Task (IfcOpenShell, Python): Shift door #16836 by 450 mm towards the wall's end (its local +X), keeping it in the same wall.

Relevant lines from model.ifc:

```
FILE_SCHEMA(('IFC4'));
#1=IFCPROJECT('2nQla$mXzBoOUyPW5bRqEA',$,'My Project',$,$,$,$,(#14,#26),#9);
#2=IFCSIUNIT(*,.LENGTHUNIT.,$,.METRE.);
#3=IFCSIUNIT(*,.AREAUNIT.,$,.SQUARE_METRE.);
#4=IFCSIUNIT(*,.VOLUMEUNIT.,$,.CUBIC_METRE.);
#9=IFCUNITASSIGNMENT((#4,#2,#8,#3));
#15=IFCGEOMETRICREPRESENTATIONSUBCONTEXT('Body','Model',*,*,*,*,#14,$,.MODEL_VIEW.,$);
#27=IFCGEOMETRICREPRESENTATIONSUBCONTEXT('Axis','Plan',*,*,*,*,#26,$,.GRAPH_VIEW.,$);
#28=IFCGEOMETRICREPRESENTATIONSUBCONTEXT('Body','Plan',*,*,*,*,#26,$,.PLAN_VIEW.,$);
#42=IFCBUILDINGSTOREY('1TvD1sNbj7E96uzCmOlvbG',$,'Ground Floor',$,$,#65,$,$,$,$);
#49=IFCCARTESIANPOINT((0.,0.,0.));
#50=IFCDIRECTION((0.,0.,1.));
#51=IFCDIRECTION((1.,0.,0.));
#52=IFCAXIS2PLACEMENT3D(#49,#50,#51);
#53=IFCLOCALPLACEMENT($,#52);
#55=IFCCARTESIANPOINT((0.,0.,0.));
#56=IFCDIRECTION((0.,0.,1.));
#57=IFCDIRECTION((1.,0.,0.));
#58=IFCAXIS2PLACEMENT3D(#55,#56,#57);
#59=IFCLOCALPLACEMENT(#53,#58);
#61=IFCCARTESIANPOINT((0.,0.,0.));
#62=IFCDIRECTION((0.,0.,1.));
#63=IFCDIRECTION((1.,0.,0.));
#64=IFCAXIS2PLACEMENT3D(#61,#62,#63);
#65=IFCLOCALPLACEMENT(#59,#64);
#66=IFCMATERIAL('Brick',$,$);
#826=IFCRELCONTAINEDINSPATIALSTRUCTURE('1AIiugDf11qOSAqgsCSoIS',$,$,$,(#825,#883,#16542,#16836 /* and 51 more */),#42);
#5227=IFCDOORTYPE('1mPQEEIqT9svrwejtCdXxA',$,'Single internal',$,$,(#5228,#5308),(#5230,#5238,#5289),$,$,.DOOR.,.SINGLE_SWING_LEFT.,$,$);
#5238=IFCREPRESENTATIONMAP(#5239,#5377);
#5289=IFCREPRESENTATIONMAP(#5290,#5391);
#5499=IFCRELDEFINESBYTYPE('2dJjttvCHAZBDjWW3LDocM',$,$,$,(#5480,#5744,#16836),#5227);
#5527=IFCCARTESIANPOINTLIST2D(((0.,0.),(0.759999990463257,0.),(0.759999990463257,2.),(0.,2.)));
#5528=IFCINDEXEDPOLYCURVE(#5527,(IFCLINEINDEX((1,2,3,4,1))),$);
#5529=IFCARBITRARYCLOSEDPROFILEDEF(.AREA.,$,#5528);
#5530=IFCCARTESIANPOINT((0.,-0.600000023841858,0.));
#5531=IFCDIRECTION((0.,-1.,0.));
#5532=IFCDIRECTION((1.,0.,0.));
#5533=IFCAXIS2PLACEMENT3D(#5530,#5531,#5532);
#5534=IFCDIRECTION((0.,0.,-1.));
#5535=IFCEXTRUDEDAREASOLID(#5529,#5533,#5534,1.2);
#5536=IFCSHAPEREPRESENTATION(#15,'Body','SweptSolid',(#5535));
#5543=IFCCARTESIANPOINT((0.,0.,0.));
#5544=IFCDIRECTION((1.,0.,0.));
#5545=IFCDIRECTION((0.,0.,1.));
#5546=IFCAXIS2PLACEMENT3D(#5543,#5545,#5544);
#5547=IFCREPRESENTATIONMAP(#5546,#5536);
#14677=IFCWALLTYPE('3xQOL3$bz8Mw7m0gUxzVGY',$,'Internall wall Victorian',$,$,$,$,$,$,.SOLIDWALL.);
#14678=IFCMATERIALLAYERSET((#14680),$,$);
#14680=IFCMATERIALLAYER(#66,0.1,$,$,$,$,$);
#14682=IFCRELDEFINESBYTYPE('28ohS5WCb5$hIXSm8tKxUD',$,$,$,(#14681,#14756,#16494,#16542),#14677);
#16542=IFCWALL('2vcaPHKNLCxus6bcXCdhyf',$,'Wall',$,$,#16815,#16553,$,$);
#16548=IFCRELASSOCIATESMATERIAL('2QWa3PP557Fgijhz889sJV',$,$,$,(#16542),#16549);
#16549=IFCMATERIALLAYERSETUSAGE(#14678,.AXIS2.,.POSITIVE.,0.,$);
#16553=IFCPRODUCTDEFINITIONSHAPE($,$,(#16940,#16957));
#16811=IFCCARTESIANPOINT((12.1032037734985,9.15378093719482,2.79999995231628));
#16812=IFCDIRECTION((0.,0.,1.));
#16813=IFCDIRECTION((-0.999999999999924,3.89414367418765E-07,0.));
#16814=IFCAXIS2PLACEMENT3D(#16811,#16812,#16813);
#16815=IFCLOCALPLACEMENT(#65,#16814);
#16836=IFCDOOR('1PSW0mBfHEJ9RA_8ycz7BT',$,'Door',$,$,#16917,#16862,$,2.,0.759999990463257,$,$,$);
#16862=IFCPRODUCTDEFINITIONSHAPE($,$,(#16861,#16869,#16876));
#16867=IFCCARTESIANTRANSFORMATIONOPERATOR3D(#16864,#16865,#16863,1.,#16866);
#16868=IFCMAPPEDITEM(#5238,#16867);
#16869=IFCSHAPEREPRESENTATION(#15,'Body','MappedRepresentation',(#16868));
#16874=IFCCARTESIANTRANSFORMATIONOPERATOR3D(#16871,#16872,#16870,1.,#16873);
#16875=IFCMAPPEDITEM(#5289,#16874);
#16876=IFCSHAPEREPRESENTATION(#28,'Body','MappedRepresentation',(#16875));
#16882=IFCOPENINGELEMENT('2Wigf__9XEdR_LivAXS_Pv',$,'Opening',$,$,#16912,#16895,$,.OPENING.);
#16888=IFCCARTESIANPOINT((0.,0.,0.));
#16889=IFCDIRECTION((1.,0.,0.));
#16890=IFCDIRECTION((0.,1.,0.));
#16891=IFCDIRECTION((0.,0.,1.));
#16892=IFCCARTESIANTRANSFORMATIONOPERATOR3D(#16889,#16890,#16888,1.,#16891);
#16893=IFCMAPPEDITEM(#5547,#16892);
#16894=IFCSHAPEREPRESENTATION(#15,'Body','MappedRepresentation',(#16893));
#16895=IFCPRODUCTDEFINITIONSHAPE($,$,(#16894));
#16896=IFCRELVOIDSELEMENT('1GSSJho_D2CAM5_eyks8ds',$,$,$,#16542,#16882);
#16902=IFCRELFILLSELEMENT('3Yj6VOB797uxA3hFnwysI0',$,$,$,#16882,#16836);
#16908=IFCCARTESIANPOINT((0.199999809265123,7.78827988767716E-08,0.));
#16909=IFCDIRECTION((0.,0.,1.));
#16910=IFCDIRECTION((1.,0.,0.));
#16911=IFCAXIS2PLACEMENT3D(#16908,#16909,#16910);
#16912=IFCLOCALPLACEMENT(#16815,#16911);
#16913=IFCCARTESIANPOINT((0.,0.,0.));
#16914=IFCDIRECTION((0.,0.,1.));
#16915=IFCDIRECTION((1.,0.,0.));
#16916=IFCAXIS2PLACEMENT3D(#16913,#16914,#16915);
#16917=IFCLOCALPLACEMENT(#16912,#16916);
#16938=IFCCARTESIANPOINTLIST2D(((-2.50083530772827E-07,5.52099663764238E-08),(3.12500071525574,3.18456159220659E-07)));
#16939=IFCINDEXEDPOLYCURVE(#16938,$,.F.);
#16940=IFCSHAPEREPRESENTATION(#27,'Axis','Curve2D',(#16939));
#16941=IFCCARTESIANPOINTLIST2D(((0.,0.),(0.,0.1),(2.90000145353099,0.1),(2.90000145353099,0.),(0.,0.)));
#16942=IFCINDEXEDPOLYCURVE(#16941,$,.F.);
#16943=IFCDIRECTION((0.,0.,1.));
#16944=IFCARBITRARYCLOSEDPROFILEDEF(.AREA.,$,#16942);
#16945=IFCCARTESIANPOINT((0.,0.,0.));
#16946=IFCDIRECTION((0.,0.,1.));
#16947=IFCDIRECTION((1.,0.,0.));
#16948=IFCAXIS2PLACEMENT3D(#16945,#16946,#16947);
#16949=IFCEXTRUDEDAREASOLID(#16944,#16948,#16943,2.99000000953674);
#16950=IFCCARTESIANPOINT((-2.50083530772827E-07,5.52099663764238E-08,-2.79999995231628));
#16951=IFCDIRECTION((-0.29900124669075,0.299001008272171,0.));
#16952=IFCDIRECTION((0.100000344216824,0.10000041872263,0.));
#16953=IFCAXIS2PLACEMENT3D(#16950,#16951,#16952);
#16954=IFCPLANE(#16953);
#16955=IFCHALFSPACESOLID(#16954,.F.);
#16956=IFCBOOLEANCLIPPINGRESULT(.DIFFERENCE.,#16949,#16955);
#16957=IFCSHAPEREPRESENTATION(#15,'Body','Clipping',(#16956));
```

```python
import ifcopenshell
import ifcopenshell.api.geometry
import ifcopenshell.util.placement
import ifcopenshell.util.unit

model = ifcopenshell.open("model.ifc")
unit_scale = ifcopenshell.util.unit.calculate_unit_scale(model)

door = model.by_guid("1PSW0mBfHEJ9RA_8ycz7BT")
opening = door.FillsVoids[0].RelatingOpeningElement
wall = opening.VoidsElements[0].RelatingBuildingElement

wall_matrix = ifcopenshell.util.placement.get_local_placement(wall.ObjectPlacement)
shift = wall_matrix[:3, 0] * 0.45 / unit_scale
before = ifcopenshell.util.placement.get_local_placement(door.ObjectPlacement)[:3, 3].copy()

# The door is placed relative to its opening, so it follows when the opening moves.
matrix = ifcopenshell.util.placement.get_local_placement(opening.ObjectPlacement)
matrix[:3, 3] += shift
ifcopenshell.api.geometry.edit_object_placement(
    model, product=opening, matrix=matrix, is_si=False, should_transform_children=True
)

after = ifcopenshell.util.placement.get_local_placement(door.ObjectPlacement)[:3, 3]
print("door moved by", (after - before).round(3) + 0.0)

model.write("model_v2.ifc")
```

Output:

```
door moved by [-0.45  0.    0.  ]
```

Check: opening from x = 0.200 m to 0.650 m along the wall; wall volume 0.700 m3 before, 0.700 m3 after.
